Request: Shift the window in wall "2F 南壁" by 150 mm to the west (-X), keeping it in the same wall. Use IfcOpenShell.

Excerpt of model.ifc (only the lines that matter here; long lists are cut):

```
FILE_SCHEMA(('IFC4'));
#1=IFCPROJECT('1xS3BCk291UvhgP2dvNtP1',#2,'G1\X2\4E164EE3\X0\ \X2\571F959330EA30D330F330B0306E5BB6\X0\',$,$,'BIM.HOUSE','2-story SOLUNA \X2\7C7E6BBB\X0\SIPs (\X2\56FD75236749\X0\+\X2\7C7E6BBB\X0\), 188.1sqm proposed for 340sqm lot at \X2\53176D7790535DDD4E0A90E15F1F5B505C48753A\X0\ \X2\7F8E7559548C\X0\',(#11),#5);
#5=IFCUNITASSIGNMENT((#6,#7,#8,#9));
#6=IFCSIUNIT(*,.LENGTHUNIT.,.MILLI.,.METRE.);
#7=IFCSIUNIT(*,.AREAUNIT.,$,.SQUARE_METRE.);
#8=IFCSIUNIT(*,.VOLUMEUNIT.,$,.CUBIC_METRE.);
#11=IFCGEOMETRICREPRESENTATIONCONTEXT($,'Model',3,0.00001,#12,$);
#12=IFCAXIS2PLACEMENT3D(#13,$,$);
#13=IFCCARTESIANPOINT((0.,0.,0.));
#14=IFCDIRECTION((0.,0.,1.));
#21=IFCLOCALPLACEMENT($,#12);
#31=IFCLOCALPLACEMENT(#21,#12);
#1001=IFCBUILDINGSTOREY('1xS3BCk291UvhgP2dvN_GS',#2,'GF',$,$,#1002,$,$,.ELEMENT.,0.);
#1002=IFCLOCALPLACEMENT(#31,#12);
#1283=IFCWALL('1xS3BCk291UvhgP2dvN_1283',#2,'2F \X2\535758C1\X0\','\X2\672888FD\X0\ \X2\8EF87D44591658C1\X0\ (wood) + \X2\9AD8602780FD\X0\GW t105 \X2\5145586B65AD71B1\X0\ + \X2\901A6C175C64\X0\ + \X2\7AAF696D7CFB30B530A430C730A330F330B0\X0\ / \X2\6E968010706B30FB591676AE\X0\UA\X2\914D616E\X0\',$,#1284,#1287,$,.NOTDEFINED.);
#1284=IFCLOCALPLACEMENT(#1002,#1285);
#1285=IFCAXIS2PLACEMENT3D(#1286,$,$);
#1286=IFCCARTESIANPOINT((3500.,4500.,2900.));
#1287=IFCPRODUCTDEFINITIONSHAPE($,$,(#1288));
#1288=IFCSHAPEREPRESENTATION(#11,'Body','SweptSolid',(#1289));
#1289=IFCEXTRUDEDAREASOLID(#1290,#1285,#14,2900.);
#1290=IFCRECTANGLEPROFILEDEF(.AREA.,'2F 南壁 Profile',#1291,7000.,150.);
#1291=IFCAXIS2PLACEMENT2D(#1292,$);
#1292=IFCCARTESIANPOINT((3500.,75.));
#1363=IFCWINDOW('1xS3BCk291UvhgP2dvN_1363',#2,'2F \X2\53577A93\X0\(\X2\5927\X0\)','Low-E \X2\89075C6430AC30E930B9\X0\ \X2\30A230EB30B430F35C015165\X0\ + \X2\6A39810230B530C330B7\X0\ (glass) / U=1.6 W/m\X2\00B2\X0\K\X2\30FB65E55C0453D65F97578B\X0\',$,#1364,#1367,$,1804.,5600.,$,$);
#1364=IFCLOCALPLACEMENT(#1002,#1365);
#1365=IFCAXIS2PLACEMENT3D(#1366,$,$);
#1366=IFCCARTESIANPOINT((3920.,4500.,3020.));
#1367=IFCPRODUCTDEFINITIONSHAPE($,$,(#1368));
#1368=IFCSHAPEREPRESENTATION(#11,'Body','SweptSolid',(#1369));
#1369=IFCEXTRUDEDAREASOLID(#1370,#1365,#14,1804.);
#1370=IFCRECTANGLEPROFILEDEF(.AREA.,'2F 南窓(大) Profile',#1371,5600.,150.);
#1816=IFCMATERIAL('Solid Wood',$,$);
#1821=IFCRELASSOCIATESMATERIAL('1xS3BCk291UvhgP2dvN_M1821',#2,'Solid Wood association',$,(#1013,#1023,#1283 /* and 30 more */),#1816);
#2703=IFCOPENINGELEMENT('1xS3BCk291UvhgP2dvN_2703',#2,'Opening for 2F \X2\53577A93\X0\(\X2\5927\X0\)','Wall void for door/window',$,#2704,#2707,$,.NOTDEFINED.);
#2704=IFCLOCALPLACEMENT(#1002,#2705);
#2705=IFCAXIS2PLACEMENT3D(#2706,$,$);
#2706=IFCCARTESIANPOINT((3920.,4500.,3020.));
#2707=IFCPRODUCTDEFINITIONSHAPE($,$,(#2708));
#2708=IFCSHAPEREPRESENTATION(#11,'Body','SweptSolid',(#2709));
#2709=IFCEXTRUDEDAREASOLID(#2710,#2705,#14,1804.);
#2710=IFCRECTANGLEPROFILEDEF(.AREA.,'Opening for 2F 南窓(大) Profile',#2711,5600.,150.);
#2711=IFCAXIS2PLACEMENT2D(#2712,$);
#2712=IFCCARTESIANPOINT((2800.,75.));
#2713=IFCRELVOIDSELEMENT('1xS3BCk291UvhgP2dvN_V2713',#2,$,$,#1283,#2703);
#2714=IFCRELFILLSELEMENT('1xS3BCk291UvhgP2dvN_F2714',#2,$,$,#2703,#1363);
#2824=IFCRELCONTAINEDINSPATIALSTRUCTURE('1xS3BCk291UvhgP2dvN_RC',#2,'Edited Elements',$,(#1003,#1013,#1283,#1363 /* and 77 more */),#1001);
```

```python
import ifcopenshell
import ifcopenshell.api.geometry
import ifcopenshell.util.placement
import ifcopenshell.util.unit

model = ifcopenshell.open("model.ifc")
unit_scale = ifcopenshell.util.unit.calculate_unit_scale(model)

window = model.by_guid("1xS3BCk291UvhgP2dvN_1363")
opening = window.FillsVoids[0].RelatingOpeningElement
wall = opening.VoidsElements[0].RelatingBuildingElement

wall_matrix = ifcopenshell.util.placement.get_local_placement(wall.ObjectPlacement)
shift = wall_matrix[:3, 0] * -0.15 / unit_scale
before = ifcopenshell.util.placement.get_local_placement(window.ObjectPlacement)[:3, 3].copy()

# The window is not placed relative to its opening, so move both.
for product in (opening, window):
    matrix = ifcopenshell.util.placement.get_local_placement(product.ObjectPlacement)
    matrix[:3, 3] += shift
    ifcopenshell.api.geometry.edit_object_placement(model, product=product, matrix=matrix, is_si=False)

after = ifcopenshell.util.placement.get_local_placement(window.ObjectPlacement)[:3, 3]
print("window moved by", (after - before).round(3) + 0.0)

model.write("model_updated.ifc")
```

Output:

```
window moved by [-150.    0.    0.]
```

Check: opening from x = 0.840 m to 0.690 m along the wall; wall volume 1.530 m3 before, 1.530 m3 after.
